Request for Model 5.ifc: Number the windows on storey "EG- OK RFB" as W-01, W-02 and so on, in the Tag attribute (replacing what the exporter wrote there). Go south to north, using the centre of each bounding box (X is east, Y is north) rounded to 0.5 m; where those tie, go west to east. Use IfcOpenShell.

First a look at what the model holds.

```python
import ifcopenshell
import ifcopenshell.util.element
import ifcopenshell.util.placement

model = ifcopenshell.open("Model 5.ifc")
print(model.schema)
storey = next(s for s in model.by_type("IfcBuildingStorey") if s.Name == "EG- OK RFB")
windows = [e for e in ifcopenshell.util.element.get_decomposition(storey) if e.is_a("IfcWindow")]
for e in sorted(windows, key=lambda e: e.id()):
    origin = ifcopenshell.util.placement.get_local_placement(e.ObjectPlacement)[:3, 3]
    print(e.id(), e.Tag, e.Name, origin.round(2) + 0.0, sep=" | ")
```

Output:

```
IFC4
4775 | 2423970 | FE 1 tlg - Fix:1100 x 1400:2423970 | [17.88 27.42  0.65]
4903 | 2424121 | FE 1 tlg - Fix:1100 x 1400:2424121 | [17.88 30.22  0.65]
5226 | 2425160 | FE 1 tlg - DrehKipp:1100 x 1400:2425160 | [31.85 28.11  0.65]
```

```python
import ifcopenshell
import ifcopenshell.geom
import ifcopenshell.util.element
import ifcopenshell.util.shape

model = ifcopenshell.open("Model 5.ifc")
settings = ifcopenshell.geom.settings()
settings.set("use-world-coords", True)


def centre(element):
    shape = ifcopenshell.geom.create_shape(settings, element)
    return ifcopenshell.util.shape.get_bbox_centroid(shape.geometry)


storey = next(s for s in model.by_type("IfcBuildingStorey") if s.Name == "EG- OK RFB")
windows = [e for e in ifcopenshell.util.element.get_decomposition(storey) if e.is_a("IfcWindow")]

# Insertion points can sit at a corner or the storey origin, so sort by the geometry (in metres).
centres = {e: centre(e) for e in windows}
windows.sort(key=lambda e: (round(centres[e][1] / 0.5), centres[e][0]))

for i, e in enumerate(windows, start=1):
    number = f"W-{i:02d}"
    e.Tag = number
    print(e.id(), number)

model.write("Model 5-out.ifc")
```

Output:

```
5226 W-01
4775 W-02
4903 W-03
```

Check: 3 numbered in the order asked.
